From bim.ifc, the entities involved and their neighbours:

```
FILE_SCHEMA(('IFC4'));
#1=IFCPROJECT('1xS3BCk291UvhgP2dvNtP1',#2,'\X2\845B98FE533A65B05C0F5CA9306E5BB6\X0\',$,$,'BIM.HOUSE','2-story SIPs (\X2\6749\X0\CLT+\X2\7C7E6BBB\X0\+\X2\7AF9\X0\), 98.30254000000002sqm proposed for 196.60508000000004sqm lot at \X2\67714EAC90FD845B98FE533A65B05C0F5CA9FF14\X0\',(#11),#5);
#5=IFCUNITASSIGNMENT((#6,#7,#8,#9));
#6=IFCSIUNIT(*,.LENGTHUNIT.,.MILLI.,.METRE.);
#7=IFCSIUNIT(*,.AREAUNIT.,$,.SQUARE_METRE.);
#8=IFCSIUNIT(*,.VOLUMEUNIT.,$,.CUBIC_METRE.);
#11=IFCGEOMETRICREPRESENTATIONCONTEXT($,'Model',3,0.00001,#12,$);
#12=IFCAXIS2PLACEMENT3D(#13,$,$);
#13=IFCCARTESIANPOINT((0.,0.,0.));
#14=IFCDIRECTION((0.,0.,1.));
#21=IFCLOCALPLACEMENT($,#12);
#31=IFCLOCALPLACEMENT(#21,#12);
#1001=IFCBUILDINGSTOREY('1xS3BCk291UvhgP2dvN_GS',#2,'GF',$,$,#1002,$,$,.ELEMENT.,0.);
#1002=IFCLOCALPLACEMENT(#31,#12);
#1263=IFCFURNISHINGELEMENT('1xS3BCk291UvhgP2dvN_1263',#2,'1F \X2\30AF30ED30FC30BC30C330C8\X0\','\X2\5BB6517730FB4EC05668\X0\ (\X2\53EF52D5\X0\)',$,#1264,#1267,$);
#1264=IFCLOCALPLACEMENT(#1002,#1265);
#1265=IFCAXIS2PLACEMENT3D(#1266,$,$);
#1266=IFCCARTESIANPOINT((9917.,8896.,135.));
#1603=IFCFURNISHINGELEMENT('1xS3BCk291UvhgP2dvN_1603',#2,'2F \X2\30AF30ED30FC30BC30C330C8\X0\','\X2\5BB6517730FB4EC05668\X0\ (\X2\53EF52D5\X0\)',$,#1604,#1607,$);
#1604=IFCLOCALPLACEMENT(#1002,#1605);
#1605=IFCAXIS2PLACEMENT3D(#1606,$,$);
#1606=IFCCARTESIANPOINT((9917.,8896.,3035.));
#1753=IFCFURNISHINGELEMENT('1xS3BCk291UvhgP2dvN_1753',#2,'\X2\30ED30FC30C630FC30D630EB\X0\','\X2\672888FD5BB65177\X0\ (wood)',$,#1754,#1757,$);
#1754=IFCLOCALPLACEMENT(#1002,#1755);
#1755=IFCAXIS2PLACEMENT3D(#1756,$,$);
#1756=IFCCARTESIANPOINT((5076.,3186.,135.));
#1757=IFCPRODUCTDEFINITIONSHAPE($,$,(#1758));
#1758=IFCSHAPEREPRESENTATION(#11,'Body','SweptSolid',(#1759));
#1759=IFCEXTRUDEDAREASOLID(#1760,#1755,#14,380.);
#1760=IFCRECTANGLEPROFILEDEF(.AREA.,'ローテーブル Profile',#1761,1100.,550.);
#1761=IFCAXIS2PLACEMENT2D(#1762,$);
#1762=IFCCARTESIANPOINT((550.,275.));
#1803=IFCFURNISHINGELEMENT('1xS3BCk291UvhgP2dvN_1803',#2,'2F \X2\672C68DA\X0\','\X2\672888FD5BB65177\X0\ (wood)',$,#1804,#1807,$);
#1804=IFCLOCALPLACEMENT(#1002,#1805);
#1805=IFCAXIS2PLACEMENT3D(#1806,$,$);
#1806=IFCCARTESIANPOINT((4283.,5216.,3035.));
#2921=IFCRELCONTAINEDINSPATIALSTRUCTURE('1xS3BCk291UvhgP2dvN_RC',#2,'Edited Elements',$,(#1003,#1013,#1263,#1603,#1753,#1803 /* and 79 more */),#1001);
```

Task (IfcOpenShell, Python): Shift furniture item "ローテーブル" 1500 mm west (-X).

```python
import ifcopenshell
import ifcopenshell.api.geometry
import ifcopenshell.util.placement
import ifcopenshell.util.unit

model = ifcopenshell.open("bim.ifc")
unit_scale = ifcopenshell.util.unit.calculate_unit_scale(model)

item = model.by_guid("1xS3BCk291UvhgP2dvN_1753")
matrix = ifcopenshell.util.placement.get_local_placement(item.ObjectPlacement)
matrix[0, 3] -= 1.5 / unit_scale
ifcopenshell.api.geometry.edit_object_placement(model, product=item, matrix=matrix, is_si=False)

print(ifcopenshell.util.placement.get_local_placement(item.ObjectPlacement).round(3) + 0.0)

model.write("bim_v2.ifc")
```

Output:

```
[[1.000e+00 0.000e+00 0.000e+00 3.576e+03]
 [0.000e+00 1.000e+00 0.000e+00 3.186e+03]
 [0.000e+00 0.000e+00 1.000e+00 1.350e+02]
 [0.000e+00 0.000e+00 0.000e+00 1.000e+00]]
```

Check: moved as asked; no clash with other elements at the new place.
